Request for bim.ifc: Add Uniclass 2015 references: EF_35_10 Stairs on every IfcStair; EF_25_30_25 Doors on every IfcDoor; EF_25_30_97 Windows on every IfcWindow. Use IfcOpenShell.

First a look at what the model holds.

```python
import ifcopenshell

model = ifcopenshell.open("bim.ifc")
print(model.schema)
print("classifications:", [c.Name for c in model.by_type("IfcClassification")])
for ifc_class in ("IfcDoor", "IfcRoof", "IfcStair", "IfcWall", "IfcWindow"):
    print(ifc_class, len(model.by_type(ifc_class)))
```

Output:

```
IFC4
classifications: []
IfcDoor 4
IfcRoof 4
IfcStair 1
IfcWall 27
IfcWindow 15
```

```python
import ifcopenshell
import ifcopenshell.api.classification

model = ifcopenshell.open("bim.ifc")

system = ifcopenshell.api.classification.add_classification(model, classification="Uniclass 2015")

codes = {
    "IfcStair": ("EF_35_10", "Stairs"),
    "IfcDoor": ("EF_25_30_25", "Doors"),
    "IfcWindow": ("EF_25_30_97", "Windows"),
}
for ifc_class, (code, name) in codes.items():
    products = model.by_type(ifc_class)
    ifcopenshell.api.classification.add_reference(
        model, products=products, classification=system, identification=code, name=name
    )
    print(code, len(products))

model.write("bim_updated.ifc")
```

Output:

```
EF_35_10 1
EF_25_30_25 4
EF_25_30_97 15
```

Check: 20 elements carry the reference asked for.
